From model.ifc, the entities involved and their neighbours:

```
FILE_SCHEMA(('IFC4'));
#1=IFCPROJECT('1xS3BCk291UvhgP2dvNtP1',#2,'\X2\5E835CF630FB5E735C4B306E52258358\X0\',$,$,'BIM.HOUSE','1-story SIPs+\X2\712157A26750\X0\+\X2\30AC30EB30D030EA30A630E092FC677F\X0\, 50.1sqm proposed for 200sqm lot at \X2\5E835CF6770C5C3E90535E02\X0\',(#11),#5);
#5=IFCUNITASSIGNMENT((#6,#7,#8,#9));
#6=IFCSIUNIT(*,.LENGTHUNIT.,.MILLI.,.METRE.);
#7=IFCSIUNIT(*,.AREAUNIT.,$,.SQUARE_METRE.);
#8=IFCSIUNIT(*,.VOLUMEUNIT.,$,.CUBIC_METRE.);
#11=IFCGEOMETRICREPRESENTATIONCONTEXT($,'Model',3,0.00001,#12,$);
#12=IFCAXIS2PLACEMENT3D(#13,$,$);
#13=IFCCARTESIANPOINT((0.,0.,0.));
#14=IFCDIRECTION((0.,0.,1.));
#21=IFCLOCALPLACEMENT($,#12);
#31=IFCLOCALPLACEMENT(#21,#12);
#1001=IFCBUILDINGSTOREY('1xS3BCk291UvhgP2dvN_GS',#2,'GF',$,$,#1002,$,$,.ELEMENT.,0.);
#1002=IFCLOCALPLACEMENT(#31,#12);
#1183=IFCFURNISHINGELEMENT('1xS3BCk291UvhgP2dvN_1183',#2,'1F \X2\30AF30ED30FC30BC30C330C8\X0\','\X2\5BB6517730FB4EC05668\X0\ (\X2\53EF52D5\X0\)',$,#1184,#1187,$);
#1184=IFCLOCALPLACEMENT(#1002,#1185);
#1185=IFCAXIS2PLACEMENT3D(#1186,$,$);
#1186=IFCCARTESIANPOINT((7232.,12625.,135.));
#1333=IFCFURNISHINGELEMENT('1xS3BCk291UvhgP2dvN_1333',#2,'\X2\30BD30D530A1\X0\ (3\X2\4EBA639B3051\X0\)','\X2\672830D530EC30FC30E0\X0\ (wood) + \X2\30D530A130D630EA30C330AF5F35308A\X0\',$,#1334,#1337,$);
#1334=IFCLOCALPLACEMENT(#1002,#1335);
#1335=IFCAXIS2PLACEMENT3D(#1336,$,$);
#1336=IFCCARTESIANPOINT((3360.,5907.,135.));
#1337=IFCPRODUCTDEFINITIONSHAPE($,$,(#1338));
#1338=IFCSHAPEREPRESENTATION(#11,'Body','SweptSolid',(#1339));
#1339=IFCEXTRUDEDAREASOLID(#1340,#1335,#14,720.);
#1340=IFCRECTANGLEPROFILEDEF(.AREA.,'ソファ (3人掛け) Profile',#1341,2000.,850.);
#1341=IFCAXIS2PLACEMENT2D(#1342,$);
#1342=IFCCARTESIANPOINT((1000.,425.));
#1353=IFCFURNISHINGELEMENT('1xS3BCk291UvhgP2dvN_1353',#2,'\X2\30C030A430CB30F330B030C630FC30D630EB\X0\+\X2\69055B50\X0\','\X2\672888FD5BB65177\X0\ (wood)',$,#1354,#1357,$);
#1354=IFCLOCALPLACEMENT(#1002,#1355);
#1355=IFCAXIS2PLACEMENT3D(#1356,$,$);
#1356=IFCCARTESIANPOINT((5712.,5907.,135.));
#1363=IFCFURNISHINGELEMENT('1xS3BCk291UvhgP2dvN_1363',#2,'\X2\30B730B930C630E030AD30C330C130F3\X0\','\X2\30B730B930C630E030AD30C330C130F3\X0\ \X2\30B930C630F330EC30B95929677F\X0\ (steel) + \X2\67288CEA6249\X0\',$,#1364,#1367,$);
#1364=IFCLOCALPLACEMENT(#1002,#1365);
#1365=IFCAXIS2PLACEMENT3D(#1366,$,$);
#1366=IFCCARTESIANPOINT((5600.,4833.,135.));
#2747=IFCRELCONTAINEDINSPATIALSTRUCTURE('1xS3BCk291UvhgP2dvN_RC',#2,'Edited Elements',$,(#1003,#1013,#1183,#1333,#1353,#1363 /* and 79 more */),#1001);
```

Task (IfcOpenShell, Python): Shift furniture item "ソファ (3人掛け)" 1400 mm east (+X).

```python
import ifcopenshell
import ifcopenshell.api.geometry
import ifcopenshell.util.placement
import ifcopenshell.util.unit

model = ifcopenshell.open("model.ifc")
unit_scale = ifcopenshell.util.unit.calculate_unit_scale(model)

item = model.by_id(1333)
matrix = ifcopenshell.util.placement.get_local_placement(item.ObjectPlacement)
matrix[0, 3] += 1.4 / unit_scale
ifcopenshell.api.geometry.edit_object_placement(model, product=item, matrix=matrix, is_si=False)

print(ifcopenshell.util.placement.get_local_placement(item.ObjectPlacement).round(3) + 0.0)

model.write("model_updated.ifc")
```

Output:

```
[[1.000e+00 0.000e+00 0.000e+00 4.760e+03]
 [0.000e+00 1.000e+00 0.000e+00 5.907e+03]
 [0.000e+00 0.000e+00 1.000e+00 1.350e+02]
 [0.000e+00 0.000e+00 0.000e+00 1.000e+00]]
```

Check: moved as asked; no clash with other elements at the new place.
